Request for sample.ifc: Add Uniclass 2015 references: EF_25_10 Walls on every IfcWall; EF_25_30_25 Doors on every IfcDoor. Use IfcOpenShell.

First a look at what the model holds.

```python
import ifcopenshell

model = ifcopenshell.open("sample.ifc")
print(model.schema)
print("classifications:", [c.Name for c in model.by_type("IfcClassification")])
for ifc_class in ("IfcDoor", "IfcRoof", "IfcStair", "IfcWall", "IfcWindow"):
    print(ifc_class, len(model.by_type(ifc_class)))
```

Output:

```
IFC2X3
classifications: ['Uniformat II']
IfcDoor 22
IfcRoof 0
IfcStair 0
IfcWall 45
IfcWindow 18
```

```python
import ifcopenshell
import ifcopenshell.api.classification

model = ifcopenshell.open("sample.ifc")

# IFC2X3 requires Source and Edition and has no link from the project to the system.
system = model.create_entity("IfcClassification", Source="NBS", Edition="2015", Name="Uniclass 2015")

codes = {
    "IfcWall": ("EF_25_10", "Walls"),
    "IfcDoor": ("EF_25_30_25", "Doors"),
}
for ifc_class, (code, name) in codes.items():
    products = model.by_type(ifc_class)
    ifcopenshell.api.classification.add_reference(
        model, products=products, classification=system, identification=code, name=name
    )
    print(code, len(products))

model.write("sample_updated.ifc")
```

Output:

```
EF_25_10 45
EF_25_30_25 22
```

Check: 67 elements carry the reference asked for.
